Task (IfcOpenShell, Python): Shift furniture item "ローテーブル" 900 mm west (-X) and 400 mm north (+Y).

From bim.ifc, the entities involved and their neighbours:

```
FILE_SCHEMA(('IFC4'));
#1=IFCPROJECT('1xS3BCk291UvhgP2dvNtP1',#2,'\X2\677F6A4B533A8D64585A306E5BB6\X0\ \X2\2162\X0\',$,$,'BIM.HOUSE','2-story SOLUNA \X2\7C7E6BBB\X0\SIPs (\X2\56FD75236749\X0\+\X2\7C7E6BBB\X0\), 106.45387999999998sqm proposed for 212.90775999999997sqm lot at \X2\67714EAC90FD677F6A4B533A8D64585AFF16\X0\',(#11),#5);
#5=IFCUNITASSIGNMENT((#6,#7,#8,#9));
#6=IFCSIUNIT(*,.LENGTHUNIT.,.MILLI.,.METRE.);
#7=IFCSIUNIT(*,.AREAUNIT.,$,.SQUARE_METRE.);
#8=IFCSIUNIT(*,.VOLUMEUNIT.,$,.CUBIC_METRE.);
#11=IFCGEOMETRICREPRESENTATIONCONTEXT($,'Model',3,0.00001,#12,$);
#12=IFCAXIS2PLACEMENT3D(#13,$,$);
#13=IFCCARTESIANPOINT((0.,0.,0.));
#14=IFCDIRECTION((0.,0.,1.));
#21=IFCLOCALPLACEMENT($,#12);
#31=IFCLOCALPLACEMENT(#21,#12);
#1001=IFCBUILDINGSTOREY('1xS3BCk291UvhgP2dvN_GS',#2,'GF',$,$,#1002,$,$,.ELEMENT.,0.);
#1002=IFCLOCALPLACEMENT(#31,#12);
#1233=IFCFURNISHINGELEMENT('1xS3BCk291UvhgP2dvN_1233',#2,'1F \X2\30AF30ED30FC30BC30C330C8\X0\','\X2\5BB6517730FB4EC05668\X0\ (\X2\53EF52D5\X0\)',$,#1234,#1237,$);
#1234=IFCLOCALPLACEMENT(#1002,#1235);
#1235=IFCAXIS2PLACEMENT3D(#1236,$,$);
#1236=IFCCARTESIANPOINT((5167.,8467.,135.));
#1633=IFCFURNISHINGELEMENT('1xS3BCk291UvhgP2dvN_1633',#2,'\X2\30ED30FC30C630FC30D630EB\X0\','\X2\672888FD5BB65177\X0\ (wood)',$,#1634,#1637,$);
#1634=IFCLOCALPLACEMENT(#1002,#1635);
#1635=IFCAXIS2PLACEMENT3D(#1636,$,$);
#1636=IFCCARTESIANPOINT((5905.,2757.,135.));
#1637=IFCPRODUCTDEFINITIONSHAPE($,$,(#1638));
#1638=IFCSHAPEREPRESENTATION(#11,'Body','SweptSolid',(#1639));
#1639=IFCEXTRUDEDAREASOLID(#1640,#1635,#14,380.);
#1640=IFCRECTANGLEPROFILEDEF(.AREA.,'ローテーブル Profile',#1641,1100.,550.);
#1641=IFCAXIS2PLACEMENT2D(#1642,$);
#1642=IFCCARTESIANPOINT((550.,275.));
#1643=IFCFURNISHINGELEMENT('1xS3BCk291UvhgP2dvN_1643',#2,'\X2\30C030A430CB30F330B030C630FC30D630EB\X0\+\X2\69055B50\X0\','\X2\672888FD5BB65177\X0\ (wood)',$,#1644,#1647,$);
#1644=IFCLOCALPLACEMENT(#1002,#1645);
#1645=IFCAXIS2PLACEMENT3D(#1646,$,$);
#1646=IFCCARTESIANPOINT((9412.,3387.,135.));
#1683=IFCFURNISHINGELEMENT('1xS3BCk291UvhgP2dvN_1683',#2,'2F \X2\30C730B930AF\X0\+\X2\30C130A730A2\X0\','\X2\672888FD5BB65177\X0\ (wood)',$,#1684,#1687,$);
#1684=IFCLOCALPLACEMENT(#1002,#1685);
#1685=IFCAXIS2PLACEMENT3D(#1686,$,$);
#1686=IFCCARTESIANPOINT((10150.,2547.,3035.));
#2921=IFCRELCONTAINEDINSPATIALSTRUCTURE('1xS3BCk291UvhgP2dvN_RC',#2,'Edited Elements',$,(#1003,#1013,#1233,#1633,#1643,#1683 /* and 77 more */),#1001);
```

```python
import ifcopenshell
import ifcopenshell.api.geometry
import ifcopenshell.util.placement

model = ifcopenshell.open("bim.ifc")

item = model.by_id(1633)
matrix = ifcopenshell.util.placement.get_local_placement(item.ObjectPlacement)
matrix[0, 3] -= 900.0
matrix[1, 3] += 400.0
ifcopenshell.api.geometry.edit_object_placement(model, product=item, matrix=matrix, is_si=False)

print(ifcopenshell.util.placement.get_local_placement(item.ObjectPlacement).round(3) + 0.0)

model.write("bim_v2.ifc")
```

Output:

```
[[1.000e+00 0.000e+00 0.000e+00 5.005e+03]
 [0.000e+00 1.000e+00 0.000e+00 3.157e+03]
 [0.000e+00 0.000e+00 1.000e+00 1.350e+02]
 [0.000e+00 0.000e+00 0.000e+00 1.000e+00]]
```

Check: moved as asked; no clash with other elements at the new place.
